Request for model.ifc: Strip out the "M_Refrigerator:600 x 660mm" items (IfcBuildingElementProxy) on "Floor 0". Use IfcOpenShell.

First a look at what the model holds.

```python
import ifcopenshell
import ifcopenshell.util.element

model = ifcopenshell.open("model.ifc")
print(model.schema)
storey = next(s for s in model.by_type("IfcBuildingStorey") if s.Name == "Floor 0")
proxies = [e for e in ifcopenshell.util.element.get_decomposition(storey) if e.is_a("IfcBuildingElementProxy")]
seen = {}
for e in proxies:
    element_type = ifcopenshell.util.element.get_type(e)
    name = element_type.Name if element_type not in (None, e) else None
    seen[name] = seen.get(name, 0) + 1
for name, count in sorted(seen.items(), key=str):
    print(count, "x", name)
```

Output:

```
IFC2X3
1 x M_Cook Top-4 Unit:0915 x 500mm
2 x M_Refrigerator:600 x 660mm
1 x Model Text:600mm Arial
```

```python
import ifcopenshell
import ifcopenshell.api.root
import ifcopenshell.util.element

model = ifcopenshell.open("model.ifc")

storey = next(s for s in model.by_type("IfcBuildingStorey") if s.Name == "Floor 0")
proxies = [e for e in ifcopenshell.util.element.get_decomposition(storey) if e.is_a("IfcBuildingElementProxy")]
targets = [e for e in proxies if (t := ifcopenshell.util.element.get_type(e)) not in (None, e) and t.Name == "M_Refrigerator:600 x 660mm"]

for e in targets:
    ifcopenshell.api.root.remove_product(model, product=e)
print(len(targets), "removed")

model.write("model_v2.ifc")
```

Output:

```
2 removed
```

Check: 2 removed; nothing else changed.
